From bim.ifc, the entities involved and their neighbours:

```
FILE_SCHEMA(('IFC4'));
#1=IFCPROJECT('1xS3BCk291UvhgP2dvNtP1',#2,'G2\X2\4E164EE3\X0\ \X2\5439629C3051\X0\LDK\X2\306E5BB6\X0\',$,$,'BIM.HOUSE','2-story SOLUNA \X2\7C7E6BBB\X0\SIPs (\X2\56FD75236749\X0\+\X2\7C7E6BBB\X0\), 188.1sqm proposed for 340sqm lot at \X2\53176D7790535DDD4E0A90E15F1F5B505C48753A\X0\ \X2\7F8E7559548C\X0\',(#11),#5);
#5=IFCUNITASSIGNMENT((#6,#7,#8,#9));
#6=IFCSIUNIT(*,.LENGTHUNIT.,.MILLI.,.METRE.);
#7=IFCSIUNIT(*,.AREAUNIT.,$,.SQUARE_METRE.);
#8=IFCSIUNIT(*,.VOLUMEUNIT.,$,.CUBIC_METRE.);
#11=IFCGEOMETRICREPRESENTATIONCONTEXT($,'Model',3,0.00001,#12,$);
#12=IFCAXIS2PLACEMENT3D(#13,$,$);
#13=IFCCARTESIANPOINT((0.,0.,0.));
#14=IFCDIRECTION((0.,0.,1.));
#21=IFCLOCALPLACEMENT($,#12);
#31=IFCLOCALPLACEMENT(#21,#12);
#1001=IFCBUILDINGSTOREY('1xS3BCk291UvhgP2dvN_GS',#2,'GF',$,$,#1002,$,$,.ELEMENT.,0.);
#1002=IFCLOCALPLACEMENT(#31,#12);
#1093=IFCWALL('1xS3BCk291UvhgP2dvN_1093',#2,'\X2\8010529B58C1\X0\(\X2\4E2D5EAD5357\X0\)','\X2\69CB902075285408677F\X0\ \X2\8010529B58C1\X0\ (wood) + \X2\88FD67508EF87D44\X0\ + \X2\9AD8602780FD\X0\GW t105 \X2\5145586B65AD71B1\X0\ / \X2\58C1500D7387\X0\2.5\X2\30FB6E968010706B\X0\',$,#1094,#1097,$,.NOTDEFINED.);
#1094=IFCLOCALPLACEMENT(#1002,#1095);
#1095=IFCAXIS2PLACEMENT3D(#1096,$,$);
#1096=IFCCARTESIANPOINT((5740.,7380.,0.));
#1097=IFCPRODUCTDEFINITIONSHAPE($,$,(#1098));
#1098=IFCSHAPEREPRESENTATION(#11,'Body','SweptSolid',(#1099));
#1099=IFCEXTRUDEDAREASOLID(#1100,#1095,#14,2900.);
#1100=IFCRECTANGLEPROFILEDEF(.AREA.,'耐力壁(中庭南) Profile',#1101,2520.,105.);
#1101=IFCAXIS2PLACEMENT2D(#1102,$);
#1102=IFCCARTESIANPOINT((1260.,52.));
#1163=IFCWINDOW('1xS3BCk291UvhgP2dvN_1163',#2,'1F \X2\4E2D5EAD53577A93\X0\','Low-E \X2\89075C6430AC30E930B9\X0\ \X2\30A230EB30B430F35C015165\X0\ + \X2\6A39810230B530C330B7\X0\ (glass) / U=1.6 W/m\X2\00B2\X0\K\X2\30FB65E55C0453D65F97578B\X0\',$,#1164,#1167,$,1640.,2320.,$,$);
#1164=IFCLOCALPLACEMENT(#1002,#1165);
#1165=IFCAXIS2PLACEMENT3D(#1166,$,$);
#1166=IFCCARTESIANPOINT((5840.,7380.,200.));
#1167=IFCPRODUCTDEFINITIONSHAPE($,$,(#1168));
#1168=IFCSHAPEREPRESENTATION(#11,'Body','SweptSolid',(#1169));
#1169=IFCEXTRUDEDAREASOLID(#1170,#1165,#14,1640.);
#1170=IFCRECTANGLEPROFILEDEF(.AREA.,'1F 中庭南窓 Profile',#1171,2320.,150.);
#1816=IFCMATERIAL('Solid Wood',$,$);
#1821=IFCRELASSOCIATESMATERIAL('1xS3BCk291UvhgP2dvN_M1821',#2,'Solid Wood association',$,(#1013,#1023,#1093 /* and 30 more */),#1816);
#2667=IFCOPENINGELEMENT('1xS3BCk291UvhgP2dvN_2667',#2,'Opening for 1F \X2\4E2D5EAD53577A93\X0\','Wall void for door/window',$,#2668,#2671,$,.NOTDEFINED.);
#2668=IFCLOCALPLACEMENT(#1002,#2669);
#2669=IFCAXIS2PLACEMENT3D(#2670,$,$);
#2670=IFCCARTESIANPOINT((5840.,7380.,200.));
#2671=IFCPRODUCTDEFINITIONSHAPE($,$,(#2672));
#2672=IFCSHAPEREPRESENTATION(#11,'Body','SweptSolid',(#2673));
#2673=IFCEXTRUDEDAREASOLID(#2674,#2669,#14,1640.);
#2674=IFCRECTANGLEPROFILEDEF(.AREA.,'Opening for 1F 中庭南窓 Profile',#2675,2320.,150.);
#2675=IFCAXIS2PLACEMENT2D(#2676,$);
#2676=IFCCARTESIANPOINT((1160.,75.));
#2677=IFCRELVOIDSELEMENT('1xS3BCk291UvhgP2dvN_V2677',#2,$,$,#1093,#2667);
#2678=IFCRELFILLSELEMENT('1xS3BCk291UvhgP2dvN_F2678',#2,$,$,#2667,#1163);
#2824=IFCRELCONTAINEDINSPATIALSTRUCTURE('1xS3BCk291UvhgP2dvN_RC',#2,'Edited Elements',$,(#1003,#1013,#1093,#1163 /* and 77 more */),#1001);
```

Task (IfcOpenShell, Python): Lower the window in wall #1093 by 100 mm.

```python
import numpy as np
import ifcopenshell
import ifcopenshell.api.geometry
import ifcopenshell.util.placement
import ifcopenshell.util.unit

model = ifcopenshell.open("bim.ifc")
unit_scale = ifcopenshell.util.unit.calculate_unit_scale(model)

window = model.by_id(1163)
opening = window.FillsVoids[0].RelatingOpeningElement
dz = -100.0

shift = np.array([0.0, 0.0, dz])
# The window is not placed relative to its opening, so move both.
for product in (opening, window):
    matrix = ifcopenshell.util.placement.get_local_placement(product.ObjectPlacement)
    matrix[:3, 3] += shift
    ifcopenshell.api.geometry.edit_object_placement(model, product=product, matrix=matrix, is_si=False)

print(f"moved by {dz * unit_scale:+.3f} m")

model.write("bim_updated.ifc")
```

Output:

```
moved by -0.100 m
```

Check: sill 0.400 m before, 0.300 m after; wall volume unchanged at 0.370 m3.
